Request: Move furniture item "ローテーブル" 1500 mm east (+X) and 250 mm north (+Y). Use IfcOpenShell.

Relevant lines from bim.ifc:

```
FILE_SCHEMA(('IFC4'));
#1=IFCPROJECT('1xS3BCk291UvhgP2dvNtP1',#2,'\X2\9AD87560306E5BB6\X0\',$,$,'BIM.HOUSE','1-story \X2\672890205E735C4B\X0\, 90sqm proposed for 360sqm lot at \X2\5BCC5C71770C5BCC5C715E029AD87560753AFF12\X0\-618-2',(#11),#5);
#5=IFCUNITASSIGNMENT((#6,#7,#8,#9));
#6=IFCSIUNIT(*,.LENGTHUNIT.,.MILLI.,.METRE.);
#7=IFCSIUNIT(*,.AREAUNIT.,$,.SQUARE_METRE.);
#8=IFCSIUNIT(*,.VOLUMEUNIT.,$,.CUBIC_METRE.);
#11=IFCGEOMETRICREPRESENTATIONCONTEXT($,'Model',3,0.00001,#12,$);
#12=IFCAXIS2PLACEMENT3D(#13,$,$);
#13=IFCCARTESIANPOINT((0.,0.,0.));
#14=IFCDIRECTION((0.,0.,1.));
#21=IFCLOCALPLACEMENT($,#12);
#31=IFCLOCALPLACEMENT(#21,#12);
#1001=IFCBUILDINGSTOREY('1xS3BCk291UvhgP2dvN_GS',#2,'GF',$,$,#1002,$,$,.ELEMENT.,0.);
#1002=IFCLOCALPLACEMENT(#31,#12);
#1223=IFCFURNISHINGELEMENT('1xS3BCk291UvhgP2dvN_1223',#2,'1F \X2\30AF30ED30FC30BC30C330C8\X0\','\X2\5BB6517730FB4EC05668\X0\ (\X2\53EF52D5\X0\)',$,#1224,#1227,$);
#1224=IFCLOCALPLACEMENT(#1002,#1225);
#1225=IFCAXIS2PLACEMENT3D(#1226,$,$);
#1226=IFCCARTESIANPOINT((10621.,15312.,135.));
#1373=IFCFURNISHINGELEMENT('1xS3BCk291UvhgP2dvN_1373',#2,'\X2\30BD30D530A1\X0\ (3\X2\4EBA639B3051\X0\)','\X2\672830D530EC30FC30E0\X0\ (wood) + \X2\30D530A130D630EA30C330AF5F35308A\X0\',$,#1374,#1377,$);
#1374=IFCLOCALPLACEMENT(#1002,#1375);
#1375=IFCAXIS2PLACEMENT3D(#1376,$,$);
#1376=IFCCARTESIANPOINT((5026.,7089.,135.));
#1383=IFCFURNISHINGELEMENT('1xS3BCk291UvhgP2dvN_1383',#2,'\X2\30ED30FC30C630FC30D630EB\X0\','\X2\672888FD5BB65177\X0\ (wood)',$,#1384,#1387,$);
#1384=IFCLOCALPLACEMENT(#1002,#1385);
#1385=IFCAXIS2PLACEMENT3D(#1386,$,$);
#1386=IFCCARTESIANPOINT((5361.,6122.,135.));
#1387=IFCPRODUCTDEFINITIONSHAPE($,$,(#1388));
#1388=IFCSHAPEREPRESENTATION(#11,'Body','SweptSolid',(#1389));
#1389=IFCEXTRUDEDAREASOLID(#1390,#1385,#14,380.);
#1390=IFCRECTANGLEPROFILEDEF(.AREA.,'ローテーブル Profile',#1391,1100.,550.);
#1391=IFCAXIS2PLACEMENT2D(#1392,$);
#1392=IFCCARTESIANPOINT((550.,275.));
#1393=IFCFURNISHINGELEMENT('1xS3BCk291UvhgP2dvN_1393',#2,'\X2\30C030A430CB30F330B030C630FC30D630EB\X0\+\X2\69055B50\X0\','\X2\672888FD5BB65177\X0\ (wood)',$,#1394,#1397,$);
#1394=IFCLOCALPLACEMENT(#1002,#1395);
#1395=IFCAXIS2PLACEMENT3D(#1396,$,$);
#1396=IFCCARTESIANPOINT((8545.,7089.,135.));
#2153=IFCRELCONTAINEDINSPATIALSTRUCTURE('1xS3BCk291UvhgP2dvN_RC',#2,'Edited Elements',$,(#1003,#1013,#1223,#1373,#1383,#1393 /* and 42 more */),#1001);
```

```python
import ifcopenshell
import ifcopenshell.api.geometry
import ifcopenshell.util.placement

model = ifcopenshell.open("bim.ifc")

item = model.by_guid("1xS3BCk291UvhgP2dvN_1383")
matrix = ifcopenshell.util.placement.get_local_placement(item.ObjectPlacement)
matrix[0, 3] += 1500.0
matrix[1, 3] += 250.0
ifcopenshell.api.geometry.edit_object_placement(model, product=item, matrix=matrix, is_si=False)

print(ifcopenshell.util.placement.get_local_placement(item.ObjectPlacement).round(3) + 0.0)

model.write("bim_updated.ifc")
```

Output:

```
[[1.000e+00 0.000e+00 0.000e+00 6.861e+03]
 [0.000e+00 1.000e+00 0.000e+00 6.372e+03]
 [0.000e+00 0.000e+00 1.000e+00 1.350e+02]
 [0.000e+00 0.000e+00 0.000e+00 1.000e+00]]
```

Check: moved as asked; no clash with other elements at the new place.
